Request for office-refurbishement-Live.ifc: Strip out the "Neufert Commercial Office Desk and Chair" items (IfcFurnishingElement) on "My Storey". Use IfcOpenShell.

First a look at what the model holds.

```python
import ifcopenshell
import ifcopenshell.util.element

model = ifcopenshell.open("office-refurbishement-Live.ifc")
print(model.schema)
storey = next(s for s in model.by_type("IfcBuildingStorey") if s.Name == "My Storey")
furniture = [e for e in ifcopenshell.util.element.get_decomposition(storey) if e.is_a("IfcFurnishingElement")]
seen = {}
for e in furniture:
    element_type = ifcopenshell.util.element.get_type(e)
    name = element_type.Name if element_type not in (None, e) else None
    seen[name] = seen.get(name, 0) + 1
for name, count in sorted(seen.items(), key=str):
    print(count, "x", name)
```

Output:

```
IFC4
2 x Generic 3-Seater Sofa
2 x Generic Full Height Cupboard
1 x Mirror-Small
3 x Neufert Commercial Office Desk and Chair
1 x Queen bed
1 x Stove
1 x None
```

```python
import ifcopenshell
import ifcopenshell.api.root
import ifcopenshell.util.element

model = ifcopenshell.open("office-refurbishement-Live.ifc")

storey = next(s for s in model.by_type("IfcBuildingStorey") if s.Name == "My Storey")
furniture = [e for e in ifcopenshell.util.element.get_decomposition(storey) if e.is_a("IfcFurnishingElement")]
targets = [e for e in furniture if (t := ifcopenshell.util.element.get_type(e)) not in (None, e) and t.Name == "Neufert Commercial Office Desk and Chair"]

for e in targets:
    ifcopenshell.api.root.remove_product(model, product=e)
print(len(targets), "removed")

model.write("office-refurbishement-Live-out.ifc")
```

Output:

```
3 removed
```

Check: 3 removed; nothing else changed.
